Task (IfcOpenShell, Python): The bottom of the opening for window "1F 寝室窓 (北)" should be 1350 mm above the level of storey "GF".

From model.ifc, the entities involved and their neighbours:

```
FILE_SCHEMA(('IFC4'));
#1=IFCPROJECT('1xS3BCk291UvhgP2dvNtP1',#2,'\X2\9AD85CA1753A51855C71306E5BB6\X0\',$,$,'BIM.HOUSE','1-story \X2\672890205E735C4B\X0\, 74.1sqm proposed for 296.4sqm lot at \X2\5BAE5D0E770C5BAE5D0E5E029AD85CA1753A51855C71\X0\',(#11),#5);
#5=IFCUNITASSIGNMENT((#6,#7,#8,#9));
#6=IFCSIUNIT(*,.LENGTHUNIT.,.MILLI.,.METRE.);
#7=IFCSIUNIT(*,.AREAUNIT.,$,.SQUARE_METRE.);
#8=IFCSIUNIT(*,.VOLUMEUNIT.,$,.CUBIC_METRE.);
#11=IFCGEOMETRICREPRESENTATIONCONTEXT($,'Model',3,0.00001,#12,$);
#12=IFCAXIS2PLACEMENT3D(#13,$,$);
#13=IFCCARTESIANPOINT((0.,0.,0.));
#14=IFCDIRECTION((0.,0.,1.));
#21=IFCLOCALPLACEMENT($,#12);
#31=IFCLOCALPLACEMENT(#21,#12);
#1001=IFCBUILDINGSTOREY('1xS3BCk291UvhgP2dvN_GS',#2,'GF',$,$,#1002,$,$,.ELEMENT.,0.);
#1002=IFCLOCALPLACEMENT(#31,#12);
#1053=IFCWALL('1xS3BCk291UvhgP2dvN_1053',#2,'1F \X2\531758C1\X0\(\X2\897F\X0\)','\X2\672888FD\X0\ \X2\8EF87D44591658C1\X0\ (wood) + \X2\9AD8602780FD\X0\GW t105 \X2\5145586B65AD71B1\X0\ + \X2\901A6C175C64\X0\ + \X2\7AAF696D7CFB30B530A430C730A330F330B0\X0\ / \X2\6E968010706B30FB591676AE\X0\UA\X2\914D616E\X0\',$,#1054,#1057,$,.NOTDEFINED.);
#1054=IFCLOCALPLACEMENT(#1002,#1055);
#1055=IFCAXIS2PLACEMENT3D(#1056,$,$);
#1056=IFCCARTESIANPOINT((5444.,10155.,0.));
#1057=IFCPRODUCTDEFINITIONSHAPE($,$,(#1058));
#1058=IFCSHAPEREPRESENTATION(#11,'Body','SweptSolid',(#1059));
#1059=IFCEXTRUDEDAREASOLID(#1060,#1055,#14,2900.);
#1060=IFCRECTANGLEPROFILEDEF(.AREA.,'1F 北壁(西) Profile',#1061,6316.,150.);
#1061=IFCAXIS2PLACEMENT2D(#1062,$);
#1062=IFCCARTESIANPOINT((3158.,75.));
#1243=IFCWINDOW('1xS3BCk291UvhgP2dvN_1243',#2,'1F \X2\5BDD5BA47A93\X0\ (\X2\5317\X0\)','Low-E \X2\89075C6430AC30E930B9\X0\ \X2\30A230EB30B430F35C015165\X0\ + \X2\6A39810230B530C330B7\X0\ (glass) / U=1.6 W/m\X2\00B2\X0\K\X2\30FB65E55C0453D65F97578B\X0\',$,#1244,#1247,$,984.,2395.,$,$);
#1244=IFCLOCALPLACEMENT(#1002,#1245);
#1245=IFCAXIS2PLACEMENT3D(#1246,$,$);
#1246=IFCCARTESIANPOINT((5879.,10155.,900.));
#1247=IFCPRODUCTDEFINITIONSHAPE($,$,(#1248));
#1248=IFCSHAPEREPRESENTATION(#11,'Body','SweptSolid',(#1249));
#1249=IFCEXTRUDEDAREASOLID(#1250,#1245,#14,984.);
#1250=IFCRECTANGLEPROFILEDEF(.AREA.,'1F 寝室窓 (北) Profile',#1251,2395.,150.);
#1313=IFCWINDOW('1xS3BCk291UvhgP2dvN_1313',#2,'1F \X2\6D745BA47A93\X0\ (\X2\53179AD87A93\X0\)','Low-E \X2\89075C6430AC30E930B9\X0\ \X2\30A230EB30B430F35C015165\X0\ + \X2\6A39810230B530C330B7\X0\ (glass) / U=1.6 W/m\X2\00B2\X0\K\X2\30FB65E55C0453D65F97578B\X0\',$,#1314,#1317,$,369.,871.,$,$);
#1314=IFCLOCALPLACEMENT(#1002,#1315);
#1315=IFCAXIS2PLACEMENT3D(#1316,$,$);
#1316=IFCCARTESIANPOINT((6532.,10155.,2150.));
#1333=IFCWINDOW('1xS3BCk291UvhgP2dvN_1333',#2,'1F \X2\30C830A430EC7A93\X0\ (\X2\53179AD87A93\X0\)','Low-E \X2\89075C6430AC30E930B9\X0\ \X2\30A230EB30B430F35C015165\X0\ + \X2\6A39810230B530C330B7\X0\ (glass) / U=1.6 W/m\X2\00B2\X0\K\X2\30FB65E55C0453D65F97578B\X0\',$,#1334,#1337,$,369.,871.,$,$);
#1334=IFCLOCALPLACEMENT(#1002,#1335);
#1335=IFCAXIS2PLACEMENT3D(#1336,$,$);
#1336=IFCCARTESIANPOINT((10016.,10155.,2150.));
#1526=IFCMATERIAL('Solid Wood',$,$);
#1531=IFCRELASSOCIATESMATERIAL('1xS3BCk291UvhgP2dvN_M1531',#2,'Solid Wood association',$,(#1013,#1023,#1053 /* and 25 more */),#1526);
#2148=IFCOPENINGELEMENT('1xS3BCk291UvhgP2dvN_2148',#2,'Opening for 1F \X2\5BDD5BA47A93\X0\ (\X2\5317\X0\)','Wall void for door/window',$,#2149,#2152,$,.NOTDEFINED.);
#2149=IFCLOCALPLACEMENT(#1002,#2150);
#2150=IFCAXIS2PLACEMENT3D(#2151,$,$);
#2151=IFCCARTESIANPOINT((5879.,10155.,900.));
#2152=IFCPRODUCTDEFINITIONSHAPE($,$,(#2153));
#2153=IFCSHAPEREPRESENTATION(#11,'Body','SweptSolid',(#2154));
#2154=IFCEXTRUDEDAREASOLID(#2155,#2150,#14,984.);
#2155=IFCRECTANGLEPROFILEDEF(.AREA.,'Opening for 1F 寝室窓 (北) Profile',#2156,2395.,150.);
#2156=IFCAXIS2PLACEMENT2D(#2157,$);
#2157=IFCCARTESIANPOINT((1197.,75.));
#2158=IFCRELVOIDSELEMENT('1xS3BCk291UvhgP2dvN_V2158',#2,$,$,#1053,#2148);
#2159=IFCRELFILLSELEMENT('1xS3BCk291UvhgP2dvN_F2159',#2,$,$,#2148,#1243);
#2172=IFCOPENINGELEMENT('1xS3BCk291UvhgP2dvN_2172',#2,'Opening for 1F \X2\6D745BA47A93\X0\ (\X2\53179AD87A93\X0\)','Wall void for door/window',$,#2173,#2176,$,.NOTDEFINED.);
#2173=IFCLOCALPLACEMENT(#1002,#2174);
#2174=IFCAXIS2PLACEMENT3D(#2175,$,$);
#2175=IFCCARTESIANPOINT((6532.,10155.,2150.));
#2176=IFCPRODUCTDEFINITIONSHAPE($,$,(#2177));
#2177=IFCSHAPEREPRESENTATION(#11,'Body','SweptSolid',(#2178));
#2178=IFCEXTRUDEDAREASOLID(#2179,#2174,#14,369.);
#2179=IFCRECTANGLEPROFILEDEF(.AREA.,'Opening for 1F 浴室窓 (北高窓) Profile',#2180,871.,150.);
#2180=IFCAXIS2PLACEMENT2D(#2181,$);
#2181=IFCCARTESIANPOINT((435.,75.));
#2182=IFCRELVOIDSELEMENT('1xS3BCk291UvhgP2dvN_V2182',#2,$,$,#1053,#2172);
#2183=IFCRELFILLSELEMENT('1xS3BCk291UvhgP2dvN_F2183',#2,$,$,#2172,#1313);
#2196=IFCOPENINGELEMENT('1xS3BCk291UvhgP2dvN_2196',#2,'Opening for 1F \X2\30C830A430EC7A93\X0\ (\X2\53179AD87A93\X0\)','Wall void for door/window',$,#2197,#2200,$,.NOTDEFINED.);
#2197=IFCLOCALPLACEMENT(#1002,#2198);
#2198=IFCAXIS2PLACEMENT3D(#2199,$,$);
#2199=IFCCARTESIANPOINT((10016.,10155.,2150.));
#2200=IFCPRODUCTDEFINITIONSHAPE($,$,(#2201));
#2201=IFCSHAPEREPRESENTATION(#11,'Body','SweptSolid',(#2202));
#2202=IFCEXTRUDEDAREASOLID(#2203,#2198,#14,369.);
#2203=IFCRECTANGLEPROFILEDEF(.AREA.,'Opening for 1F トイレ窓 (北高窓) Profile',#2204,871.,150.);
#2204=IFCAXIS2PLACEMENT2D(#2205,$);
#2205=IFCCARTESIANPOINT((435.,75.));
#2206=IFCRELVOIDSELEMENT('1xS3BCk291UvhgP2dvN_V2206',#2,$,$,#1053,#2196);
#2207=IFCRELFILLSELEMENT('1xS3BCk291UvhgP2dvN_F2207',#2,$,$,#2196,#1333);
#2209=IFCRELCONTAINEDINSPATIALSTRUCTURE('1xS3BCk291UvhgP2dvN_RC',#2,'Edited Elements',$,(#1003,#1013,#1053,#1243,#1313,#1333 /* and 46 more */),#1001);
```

```python
import numpy as np
import ifcopenshell
import ifcopenshell.api.geometry
import ifcopenshell.geom
import ifcopenshell.util.element
import ifcopenshell.util.placement
import ifcopenshell.util.shape
import ifcopenshell.util.unit

model = ifcopenshell.open("model.ifc")
unit_scale = ifcopenshell.util.unit.calculate_unit_scale(model)

window = model.by_guid("1xS3BCk291UvhgP2dvN_1243")
opening = window.FillsVoids[0].RelatingOpeningElement
storey = ifcopenshell.util.element.get_container(window, ifc_class="IfcBuildingStorey")
level = ifcopenshell.util.placement.get_local_placement(storey.ObjectPlacement)[2, 3]

# The opening's origin need not be at the sill, so measure its lowest point.
shape = ifcopenshell.geom.create_shape(ifcopenshell.geom.settings(), opening)
bottom = ifcopenshell.util.shape.get_shape_bottom_elevation(shape, shape.geometry) / unit_scale
dz = level + 1.35 / unit_scale - bottom

shift = np.array([0.0, 0.0, dz])
# The window is not placed relative to its opening, so move both.
for product in (opening, window):
    matrix = ifcopenshell.util.placement.get_local_placement(product.ObjectPlacement)
    matrix[:3, 3] += shift
    ifcopenshell.api.geometry.edit_object_placement(model, product=product, matrix=matrix, is_si=False)

print(f"moved by {dz * unit_scale:+.3f} m")

model.write("model_edited.ifc")
```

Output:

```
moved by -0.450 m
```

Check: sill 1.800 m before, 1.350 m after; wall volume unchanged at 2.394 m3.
